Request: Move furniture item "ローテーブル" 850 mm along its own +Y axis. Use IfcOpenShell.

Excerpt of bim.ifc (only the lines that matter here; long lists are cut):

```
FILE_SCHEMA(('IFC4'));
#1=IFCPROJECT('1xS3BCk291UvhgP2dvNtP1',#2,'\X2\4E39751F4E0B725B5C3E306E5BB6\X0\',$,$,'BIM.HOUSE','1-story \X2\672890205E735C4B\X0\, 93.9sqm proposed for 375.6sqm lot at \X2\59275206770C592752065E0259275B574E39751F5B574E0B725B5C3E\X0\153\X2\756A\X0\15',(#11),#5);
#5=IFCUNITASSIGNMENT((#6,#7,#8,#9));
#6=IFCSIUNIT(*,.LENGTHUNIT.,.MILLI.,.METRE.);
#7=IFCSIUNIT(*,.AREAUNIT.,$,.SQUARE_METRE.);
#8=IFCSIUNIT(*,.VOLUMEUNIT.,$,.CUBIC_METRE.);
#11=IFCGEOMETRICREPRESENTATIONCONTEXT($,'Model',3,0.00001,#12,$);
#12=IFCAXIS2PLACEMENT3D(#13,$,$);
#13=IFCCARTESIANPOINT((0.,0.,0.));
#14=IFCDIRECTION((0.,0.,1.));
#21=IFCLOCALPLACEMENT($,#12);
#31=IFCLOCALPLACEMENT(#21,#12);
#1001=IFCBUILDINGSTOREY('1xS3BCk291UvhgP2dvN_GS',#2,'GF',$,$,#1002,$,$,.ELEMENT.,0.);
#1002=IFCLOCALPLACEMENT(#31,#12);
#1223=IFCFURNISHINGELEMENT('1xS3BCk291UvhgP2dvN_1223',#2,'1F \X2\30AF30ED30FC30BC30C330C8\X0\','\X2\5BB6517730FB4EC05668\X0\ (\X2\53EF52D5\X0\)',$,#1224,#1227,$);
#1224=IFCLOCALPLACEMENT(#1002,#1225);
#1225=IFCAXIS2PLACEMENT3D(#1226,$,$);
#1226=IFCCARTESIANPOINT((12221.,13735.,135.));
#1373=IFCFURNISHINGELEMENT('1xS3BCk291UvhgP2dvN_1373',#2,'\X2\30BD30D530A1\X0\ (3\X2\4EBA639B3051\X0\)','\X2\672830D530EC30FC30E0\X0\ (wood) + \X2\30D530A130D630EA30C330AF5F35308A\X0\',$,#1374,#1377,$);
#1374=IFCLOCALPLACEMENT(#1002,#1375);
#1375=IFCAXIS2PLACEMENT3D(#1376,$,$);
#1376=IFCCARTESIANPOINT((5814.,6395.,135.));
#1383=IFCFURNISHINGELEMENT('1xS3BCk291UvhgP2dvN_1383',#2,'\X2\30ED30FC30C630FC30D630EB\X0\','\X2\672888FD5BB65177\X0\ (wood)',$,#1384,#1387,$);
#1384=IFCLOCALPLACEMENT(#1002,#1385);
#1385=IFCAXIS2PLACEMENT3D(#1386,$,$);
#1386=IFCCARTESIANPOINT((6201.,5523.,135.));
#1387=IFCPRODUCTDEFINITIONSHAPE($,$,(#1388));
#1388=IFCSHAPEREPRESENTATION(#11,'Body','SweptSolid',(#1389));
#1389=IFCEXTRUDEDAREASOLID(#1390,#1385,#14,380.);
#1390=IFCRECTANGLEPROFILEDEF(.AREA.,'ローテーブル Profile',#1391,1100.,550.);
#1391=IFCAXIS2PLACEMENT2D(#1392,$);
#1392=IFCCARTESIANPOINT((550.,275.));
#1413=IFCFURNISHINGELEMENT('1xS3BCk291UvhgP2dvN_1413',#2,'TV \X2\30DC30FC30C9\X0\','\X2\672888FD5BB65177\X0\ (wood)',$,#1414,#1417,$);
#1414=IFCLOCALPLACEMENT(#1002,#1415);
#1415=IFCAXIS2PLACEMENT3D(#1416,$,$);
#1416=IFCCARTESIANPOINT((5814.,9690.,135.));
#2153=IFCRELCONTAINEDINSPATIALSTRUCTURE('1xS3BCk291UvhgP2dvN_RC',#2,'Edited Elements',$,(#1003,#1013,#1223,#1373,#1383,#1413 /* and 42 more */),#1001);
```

```python
import ifcopenshell
import ifcopenshell.api.geometry
import ifcopenshell.util.placement
import ifcopenshell.util.unit

model = ifcopenshell.open("bim.ifc")
unit_scale = ifcopenshell.util.unit.calculate_unit_scale(model)

item = model.by_guid("1xS3BCk291UvhgP2dvN_1383")
matrix = ifcopenshell.util.placement.get_local_placement(item.ObjectPlacement)
matrix[:3, 3] += matrix[:3, 1] * 0.85 / unit_scale
ifcopenshell.api.geometry.edit_object_placement(model, product=item, matrix=matrix, is_si=False)

print(ifcopenshell.util.placement.get_local_placement(item.ObjectPlacement).round(3) + 0.0)

model.write("bim_updated.ifc")
```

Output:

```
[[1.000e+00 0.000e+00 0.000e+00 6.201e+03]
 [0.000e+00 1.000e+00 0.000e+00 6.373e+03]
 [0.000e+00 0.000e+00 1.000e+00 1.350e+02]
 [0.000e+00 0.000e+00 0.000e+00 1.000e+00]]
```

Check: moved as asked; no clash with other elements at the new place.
